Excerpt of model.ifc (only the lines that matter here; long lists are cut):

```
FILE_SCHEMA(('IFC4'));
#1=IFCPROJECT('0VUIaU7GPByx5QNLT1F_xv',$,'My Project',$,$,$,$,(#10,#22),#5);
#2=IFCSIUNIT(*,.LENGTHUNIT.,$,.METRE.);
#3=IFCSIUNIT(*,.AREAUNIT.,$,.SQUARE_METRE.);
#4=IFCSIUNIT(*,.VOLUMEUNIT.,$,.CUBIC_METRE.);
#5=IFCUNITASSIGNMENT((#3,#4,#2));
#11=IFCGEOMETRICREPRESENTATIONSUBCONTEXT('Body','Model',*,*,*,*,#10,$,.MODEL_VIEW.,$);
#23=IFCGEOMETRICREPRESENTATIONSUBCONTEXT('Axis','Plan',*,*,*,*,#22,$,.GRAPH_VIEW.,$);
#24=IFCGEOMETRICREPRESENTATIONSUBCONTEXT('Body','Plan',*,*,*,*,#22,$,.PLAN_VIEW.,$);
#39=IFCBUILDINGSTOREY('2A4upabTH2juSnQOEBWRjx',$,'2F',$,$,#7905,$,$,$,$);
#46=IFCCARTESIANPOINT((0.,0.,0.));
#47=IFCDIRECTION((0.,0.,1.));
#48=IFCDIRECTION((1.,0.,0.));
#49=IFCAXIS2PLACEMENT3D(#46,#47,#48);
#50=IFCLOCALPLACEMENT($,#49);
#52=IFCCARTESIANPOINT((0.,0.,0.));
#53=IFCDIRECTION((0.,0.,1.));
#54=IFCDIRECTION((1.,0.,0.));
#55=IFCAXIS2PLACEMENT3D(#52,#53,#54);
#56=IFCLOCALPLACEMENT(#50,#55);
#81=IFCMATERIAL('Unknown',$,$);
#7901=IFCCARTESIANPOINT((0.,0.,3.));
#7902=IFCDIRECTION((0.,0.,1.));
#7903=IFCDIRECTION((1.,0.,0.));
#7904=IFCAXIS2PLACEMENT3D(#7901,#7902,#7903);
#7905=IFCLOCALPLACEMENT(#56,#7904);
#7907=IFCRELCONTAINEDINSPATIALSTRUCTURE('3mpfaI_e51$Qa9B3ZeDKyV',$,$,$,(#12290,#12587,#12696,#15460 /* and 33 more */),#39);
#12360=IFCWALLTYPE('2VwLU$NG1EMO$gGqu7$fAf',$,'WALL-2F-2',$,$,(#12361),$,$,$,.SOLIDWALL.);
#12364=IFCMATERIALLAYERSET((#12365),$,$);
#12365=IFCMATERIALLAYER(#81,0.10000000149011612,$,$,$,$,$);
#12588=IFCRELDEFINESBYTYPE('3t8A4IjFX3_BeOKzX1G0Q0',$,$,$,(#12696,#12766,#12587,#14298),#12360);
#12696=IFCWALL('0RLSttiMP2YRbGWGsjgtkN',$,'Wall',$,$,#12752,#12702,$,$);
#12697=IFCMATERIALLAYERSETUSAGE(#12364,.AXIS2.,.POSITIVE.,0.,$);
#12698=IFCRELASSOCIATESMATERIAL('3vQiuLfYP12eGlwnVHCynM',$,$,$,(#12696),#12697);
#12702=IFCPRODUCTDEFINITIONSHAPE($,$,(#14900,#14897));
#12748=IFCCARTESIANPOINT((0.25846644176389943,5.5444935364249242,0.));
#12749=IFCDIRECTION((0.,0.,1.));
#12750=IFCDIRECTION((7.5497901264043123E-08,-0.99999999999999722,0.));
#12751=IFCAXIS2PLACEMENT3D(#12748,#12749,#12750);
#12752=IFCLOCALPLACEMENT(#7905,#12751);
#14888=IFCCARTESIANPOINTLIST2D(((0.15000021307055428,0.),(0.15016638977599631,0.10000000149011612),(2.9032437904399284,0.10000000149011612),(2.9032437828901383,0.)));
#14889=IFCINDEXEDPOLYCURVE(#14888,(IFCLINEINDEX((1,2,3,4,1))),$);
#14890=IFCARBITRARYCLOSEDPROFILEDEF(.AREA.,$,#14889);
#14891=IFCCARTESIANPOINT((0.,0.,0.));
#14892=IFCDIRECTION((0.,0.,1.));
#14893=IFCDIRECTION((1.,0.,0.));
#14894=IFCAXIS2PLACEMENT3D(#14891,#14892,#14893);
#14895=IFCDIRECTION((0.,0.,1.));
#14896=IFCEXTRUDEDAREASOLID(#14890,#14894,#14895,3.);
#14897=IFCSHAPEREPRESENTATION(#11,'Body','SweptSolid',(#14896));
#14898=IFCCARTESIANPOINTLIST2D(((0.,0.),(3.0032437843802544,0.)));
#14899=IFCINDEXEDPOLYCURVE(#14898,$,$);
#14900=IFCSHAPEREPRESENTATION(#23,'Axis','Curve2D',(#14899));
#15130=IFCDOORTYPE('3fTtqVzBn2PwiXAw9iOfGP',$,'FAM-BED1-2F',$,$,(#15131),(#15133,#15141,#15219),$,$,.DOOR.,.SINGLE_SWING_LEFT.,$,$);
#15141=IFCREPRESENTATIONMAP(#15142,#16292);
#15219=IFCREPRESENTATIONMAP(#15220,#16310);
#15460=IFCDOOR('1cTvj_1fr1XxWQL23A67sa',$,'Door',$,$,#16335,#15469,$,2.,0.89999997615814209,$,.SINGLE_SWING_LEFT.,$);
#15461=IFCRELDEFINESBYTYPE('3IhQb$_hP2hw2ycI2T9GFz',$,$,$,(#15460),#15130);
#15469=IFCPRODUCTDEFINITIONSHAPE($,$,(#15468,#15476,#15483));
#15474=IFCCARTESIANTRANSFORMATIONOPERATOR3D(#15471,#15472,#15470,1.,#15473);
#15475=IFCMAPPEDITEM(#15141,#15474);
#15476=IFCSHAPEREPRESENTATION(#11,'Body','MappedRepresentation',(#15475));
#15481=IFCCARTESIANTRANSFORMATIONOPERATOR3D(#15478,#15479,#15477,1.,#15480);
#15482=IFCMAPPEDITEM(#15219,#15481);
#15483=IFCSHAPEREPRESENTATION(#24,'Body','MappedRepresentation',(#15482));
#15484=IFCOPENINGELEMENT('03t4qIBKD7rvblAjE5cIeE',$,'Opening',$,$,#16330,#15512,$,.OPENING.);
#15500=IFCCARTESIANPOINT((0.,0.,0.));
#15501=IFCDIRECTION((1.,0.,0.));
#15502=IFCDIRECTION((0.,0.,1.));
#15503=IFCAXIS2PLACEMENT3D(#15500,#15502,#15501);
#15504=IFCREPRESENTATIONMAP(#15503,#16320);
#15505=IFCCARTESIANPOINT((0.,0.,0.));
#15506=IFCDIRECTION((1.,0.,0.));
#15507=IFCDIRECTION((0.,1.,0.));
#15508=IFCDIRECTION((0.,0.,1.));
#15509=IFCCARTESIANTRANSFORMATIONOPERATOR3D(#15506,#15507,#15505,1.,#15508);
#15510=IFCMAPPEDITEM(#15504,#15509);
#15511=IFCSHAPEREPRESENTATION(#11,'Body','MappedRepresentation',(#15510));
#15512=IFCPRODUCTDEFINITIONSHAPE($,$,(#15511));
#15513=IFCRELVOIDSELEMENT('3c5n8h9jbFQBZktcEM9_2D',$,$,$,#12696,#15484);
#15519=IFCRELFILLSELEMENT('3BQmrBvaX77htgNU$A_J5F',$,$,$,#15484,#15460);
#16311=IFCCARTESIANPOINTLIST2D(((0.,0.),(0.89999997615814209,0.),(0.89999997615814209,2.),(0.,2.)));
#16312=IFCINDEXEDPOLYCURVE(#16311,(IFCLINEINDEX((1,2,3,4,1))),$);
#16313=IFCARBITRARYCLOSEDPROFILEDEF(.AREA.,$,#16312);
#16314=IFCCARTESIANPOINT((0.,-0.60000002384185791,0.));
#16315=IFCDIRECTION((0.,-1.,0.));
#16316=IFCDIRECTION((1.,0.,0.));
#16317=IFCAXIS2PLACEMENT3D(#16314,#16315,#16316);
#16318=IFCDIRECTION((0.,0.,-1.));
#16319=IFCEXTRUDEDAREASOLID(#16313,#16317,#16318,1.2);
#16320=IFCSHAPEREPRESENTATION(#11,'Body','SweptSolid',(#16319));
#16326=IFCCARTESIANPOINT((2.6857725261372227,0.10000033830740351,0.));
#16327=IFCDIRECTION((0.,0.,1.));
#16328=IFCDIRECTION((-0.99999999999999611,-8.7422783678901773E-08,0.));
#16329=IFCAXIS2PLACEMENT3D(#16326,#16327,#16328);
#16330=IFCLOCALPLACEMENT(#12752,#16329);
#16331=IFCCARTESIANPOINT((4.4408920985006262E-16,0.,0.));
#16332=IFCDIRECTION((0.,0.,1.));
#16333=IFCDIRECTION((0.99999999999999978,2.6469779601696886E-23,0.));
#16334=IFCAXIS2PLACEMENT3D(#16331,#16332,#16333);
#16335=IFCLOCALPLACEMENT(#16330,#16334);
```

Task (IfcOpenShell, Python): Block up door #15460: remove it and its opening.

```python
import ifcopenshell
import ifcopenshell.api.feature
import ifcopenshell.api.root
import ifcopenshell.geom
import ifcopenshell.util.shape

model = ifcopenshell.open("model.ifc")
settings = ifcopenshell.geom.settings()


def volume(element):
    """Net volume in cubic metres, openings subtracted."""
    shape = ifcopenshell.geom.create_shape(settings, element)
    return ifcopenshell.util.shape.get_volume(shape.geometry)


door = model.by_guid("1cTvj_1fr1XxWQL23A67sa")
opening = door.FillsVoids[0].RelatingOpeningElement
wall = opening.VoidsElements[0].RelatingBuildingElement
before = volume(wall)

ifcopenshell.api.root.remove_product(model, product=door)
ifcopenshell.api.feature.remove_feature(model, feature=opening)

after = volume(wall)

print(f"wall volume {before:.3f} -> {after:.3f} m3")

model.write("model_edited.ifc")
```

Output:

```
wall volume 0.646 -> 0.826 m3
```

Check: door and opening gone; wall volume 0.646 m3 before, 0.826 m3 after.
